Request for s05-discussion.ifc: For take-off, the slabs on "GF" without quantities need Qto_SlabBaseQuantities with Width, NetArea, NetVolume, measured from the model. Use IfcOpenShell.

First a look at what the model holds.

```python
import ifcopenshell
import ifcopenshell.util.element
import ifcopenshell.util.unit

model = ifcopenshell.open("s05-discussion.ifc")
print(model.schema)
for unit_type in ("LENGTHUNIT", "AREAUNIT", "VOLUMEUNIT"):
    print(unit_type, ifcopenshell.util.unit.calculate_unit_scale(model, unit_type))
storey = next(s for s in model.by_type("IfcBuildingStorey") if s.Name == "GF")
slabs = [e for e in ifcopenshell.util.element.get_decomposition(storey) if e.is_a("IfcSlab")]
for e in sorted(slabs, key=lambda e: e.id()):
    print(e.id(), e.is_a(), e.Name, list(ifcopenshell.util.element.get_psets(e, qtos_only=True)), sep=" | ")
```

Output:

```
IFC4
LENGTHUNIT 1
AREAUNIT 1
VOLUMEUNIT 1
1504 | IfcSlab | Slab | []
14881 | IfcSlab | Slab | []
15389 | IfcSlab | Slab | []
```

```python
import ifcopenshell
import ifcopenshell.api.pset
import ifcopenshell.geom
import ifcopenshell.util.element
import ifcopenshell.util.shape
import ifcopenshell.util.unit

model = ifcopenshell.open("s05-discussion.ifc")
unit_scale = ifcopenshell.util.unit.calculate_unit_scale(model)
area_scale = ifcopenshell.util.unit.calculate_unit_scale(model, "AREAUNIT")
volume_scale = ifcopenshell.util.unit.calculate_unit_scale(model, "VOLUMEUNIT")
settings = ifcopenshell.geom.settings()

storey = next(s for s in model.by_type("IfcBuildingStorey") if s.Name == "GF")
slabs = [e for e in ifcopenshell.util.element.get_decomposition(storey) if e.is_a("IfcSlab")]

for e in sorted(slabs, key=lambda e: e.id()):
    if ifcopenshell.util.element.get_psets(e, qtos_only=True, should_inherit=False):
        continue
    # Geometry comes back in metres, in the element's own axes.
    shape = ifcopenshell.geom.create_shape(settings, e)
    values = {
        "Width": ifcopenshell.util.shape.get_z(shape.geometry) / unit_scale,
        "NetArea": ifcopenshell.util.shape.get_footprint_area(shape.geometry) / area_scale,
        "NetVolume": ifcopenshell.util.shape.get_volume(shape.geometry) / volume_scale,
    }
    qto = ifcopenshell.api.pset.add_qto(model, product=e, name="Qto_SlabBaseQuantities")
    ifcopenshell.api.pset.edit_qto(model, qto=qto, properties=values)
    print(e.id(), {k: round(v, 3) for k, v in values.items()})

model.write("s05-discussion_v2.ifc")
```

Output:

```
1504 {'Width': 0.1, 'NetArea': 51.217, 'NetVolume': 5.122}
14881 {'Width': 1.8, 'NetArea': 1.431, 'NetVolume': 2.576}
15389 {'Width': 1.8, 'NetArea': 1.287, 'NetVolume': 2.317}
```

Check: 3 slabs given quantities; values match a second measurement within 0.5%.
